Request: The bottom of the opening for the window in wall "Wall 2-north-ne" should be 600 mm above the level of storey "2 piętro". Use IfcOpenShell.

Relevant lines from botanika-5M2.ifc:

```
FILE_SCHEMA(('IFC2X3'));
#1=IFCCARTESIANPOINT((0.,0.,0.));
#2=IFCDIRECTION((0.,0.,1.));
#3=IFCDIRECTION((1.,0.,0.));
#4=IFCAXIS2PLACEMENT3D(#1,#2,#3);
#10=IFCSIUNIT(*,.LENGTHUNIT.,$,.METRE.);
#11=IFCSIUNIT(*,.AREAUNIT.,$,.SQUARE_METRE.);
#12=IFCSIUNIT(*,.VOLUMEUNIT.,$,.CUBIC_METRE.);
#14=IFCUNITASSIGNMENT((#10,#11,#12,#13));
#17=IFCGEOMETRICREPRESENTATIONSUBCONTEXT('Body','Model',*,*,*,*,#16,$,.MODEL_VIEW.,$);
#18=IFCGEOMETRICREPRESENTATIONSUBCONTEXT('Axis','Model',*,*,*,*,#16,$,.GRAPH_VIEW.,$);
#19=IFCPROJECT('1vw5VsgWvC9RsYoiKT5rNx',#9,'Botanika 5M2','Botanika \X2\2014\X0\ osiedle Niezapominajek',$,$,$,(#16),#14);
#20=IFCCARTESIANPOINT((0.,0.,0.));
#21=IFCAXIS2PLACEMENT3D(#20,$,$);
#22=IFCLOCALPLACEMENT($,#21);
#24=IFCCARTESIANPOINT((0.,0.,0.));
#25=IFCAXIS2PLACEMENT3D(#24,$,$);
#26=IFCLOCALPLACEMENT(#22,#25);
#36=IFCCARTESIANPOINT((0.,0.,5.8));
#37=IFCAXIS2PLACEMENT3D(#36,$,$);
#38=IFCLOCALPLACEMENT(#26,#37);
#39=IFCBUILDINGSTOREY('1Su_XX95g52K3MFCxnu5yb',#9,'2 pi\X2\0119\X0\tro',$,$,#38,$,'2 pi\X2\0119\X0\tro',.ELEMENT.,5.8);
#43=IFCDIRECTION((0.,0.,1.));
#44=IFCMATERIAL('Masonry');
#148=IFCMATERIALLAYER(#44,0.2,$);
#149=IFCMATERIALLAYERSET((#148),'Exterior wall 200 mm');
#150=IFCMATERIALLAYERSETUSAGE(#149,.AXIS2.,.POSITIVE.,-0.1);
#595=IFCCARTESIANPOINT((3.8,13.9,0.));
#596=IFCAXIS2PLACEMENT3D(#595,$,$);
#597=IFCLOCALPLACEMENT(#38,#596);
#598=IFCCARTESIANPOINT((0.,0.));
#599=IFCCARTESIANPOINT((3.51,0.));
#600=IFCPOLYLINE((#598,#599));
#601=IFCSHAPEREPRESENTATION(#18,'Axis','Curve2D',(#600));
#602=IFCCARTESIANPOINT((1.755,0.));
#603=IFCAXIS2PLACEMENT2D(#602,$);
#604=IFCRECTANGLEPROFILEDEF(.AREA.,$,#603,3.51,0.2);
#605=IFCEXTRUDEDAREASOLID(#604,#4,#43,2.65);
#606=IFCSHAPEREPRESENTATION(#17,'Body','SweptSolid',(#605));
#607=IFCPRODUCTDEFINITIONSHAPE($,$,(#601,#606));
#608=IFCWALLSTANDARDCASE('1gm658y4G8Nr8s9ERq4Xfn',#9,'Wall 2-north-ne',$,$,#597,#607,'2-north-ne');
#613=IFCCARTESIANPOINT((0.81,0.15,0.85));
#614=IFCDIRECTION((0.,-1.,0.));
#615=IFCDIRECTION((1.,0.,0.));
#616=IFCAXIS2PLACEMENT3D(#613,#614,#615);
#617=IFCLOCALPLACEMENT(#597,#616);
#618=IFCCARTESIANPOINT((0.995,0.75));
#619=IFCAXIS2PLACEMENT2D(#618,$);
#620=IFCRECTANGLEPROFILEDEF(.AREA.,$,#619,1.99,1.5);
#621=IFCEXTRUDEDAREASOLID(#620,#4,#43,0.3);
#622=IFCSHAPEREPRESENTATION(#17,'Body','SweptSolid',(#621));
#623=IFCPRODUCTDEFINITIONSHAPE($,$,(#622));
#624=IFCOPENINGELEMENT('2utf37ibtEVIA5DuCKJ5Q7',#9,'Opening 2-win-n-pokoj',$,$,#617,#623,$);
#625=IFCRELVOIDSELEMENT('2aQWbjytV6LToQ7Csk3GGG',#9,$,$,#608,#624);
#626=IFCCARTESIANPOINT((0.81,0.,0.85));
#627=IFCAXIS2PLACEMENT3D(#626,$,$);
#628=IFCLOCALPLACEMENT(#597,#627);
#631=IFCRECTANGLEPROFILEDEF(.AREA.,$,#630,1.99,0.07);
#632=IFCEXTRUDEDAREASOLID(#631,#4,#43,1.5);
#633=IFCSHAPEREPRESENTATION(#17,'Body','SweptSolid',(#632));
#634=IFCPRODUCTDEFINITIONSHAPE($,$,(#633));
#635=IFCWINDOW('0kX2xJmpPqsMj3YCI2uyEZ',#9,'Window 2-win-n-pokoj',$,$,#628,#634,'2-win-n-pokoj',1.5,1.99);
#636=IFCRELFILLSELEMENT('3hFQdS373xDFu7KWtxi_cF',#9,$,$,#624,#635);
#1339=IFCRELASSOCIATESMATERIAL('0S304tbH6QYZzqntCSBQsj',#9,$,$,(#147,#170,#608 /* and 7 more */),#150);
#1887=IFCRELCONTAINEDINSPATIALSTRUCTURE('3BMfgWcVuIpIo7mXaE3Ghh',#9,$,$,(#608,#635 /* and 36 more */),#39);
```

```python
import numpy as np
import ifcopenshell
import ifcopenshell.api.geometry
import ifcopenshell.geom
import ifcopenshell.util.element
import ifcopenshell.util.placement
import ifcopenshell.util.shape
import ifcopenshell.util.unit

model = ifcopenshell.open("botanika-5M2.ifc")
unit_scale = ifcopenshell.util.unit.calculate_unit_scale(model)

window = model.by_id(635)
opening = window.FillsVoids[0].RelatingOpeningElement
storey = ifcopenshell.util.element.get_container(window, ifc_class="IfcBuildingStorey")
level = ifcopenshell.util.placement.get_local_placement(storey.ObjectPlacement)[2, 3]

# The opening's origin need not be at the sill, so measure its lowest point.
shape = ifcopenshell.geom.create_shape(ifcopenshell.geom.settings(), opening)
bottom = ifcopenshell.util.shape.get_shape_bottom_elevation(shape, shape.geometry) / unit_scale
dz = level + 0.6 - bottom

shift = np.array([0.0, 0.0, dz])
# The window is not placed relative to its opening, so move both.
for product in (opening, window):
    matrix = ifcopenshell.util.placement.get_local_placement(product.ObjectPlacement)
    matrix[:3, 3] += shift
    ifcopenshell.api.geometry.edit_object_placement(model, product=product, matrix=matrix, is_si=False)

print(f"moved by {dz * unit_scale:+.3f} m")

model.write("botanika-5M2_edited.ifc")
```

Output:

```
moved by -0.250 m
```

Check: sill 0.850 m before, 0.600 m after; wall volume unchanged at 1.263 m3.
